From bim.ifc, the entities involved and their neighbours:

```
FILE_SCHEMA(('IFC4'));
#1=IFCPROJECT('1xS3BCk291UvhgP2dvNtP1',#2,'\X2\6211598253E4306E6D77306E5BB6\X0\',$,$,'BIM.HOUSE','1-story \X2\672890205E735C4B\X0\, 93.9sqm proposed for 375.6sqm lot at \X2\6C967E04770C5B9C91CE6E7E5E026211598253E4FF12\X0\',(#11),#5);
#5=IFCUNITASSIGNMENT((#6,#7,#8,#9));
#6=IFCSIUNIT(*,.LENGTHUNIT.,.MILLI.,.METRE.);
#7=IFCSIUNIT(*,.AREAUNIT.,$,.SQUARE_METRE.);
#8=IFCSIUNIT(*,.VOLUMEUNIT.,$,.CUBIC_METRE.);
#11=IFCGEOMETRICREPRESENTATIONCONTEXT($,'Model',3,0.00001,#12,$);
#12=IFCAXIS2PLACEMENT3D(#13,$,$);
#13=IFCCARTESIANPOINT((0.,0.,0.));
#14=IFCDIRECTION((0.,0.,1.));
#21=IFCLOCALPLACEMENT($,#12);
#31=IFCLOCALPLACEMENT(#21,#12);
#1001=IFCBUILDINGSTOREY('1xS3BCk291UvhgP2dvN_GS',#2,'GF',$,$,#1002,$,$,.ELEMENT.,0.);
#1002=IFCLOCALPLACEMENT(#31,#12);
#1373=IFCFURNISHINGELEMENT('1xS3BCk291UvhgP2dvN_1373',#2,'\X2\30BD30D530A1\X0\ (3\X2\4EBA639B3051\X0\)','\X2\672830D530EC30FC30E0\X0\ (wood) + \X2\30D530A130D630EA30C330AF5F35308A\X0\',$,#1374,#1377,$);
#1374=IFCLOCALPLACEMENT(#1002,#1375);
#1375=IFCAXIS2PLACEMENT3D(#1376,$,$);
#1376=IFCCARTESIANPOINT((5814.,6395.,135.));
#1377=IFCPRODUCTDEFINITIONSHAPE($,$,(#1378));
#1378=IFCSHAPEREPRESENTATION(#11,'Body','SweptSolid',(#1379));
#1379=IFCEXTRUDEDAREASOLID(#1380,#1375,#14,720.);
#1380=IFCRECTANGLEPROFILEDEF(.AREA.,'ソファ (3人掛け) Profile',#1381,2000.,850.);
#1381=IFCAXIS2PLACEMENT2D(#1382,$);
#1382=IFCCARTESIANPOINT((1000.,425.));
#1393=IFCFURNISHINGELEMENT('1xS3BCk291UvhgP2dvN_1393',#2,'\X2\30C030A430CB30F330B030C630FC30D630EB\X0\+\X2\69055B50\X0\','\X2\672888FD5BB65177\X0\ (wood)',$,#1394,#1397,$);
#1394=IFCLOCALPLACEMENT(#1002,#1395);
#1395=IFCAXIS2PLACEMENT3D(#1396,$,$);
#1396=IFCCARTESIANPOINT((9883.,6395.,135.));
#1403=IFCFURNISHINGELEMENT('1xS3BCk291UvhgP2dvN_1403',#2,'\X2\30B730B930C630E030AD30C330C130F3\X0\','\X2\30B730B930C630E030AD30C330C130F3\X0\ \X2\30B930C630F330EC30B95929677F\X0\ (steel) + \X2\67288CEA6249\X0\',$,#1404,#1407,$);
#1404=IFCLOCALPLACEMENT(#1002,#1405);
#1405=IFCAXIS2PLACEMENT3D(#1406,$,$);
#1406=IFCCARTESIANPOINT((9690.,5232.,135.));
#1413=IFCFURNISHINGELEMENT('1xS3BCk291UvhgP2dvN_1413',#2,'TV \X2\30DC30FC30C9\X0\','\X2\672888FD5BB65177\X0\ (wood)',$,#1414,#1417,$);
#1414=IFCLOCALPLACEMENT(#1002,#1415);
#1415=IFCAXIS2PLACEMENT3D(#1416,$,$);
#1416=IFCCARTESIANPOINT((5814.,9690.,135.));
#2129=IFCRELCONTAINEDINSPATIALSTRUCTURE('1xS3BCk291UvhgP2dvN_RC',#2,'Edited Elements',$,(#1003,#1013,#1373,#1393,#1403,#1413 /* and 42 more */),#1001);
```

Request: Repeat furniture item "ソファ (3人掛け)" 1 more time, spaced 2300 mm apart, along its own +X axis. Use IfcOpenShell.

```python
import ifcopenshell
import ifcopenshell.api.geometry
import ifcopenshell.api.root
import ifcopenshell.util.element
import ifcopenshell.util.placement

model = ifcopenshell.open("bim.ifc")


def reuse_history(source, copy):
    """copy_class also copies each property set's owner history, people and application; keep the originals."""
    for rel in copy.IsDefinedBy:
        if rel.is_a("IfcRelDefinesByProperties") and (history := rel.RelatingPropertyDefinition.OwnerHistory):
            rel.RelatingPropertyDefinition.OwnerHistory = source.OwnerHistory
            ifcopenshell.util.element.remove_deep2(model, history)


source = model.by_guid("1xS3BCk291UvhgP2dvN_1373")
base = ifcopenshell.util.placement.get_local_placement(source.ObjectPlacement)
step = base[:3, 0] * 2300.0

for i in range(1, 2):
    copy = ifcopenshell.api.root.copy_class(model, product=source)
    copy.Representation = ifcopenshell.util.element.copy_deep(
        model, source.Representation, exclude=["IfcGeometricRepresentationContext", "IfcRepresentationMap"]
    )
    reuse_history(source, copy)
    matrix = base.copy()
    matrix[:3, 3] += i * step
    print("added at", matrix[:3, 3].round(3) + 0.0)
    ifcopenshell.api.geometry.edit_object_placement(model, product=copy, matrix=matrix, is_si=False)

model.write("bim-out.ifc")
```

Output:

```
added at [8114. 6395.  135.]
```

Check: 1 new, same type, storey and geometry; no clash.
